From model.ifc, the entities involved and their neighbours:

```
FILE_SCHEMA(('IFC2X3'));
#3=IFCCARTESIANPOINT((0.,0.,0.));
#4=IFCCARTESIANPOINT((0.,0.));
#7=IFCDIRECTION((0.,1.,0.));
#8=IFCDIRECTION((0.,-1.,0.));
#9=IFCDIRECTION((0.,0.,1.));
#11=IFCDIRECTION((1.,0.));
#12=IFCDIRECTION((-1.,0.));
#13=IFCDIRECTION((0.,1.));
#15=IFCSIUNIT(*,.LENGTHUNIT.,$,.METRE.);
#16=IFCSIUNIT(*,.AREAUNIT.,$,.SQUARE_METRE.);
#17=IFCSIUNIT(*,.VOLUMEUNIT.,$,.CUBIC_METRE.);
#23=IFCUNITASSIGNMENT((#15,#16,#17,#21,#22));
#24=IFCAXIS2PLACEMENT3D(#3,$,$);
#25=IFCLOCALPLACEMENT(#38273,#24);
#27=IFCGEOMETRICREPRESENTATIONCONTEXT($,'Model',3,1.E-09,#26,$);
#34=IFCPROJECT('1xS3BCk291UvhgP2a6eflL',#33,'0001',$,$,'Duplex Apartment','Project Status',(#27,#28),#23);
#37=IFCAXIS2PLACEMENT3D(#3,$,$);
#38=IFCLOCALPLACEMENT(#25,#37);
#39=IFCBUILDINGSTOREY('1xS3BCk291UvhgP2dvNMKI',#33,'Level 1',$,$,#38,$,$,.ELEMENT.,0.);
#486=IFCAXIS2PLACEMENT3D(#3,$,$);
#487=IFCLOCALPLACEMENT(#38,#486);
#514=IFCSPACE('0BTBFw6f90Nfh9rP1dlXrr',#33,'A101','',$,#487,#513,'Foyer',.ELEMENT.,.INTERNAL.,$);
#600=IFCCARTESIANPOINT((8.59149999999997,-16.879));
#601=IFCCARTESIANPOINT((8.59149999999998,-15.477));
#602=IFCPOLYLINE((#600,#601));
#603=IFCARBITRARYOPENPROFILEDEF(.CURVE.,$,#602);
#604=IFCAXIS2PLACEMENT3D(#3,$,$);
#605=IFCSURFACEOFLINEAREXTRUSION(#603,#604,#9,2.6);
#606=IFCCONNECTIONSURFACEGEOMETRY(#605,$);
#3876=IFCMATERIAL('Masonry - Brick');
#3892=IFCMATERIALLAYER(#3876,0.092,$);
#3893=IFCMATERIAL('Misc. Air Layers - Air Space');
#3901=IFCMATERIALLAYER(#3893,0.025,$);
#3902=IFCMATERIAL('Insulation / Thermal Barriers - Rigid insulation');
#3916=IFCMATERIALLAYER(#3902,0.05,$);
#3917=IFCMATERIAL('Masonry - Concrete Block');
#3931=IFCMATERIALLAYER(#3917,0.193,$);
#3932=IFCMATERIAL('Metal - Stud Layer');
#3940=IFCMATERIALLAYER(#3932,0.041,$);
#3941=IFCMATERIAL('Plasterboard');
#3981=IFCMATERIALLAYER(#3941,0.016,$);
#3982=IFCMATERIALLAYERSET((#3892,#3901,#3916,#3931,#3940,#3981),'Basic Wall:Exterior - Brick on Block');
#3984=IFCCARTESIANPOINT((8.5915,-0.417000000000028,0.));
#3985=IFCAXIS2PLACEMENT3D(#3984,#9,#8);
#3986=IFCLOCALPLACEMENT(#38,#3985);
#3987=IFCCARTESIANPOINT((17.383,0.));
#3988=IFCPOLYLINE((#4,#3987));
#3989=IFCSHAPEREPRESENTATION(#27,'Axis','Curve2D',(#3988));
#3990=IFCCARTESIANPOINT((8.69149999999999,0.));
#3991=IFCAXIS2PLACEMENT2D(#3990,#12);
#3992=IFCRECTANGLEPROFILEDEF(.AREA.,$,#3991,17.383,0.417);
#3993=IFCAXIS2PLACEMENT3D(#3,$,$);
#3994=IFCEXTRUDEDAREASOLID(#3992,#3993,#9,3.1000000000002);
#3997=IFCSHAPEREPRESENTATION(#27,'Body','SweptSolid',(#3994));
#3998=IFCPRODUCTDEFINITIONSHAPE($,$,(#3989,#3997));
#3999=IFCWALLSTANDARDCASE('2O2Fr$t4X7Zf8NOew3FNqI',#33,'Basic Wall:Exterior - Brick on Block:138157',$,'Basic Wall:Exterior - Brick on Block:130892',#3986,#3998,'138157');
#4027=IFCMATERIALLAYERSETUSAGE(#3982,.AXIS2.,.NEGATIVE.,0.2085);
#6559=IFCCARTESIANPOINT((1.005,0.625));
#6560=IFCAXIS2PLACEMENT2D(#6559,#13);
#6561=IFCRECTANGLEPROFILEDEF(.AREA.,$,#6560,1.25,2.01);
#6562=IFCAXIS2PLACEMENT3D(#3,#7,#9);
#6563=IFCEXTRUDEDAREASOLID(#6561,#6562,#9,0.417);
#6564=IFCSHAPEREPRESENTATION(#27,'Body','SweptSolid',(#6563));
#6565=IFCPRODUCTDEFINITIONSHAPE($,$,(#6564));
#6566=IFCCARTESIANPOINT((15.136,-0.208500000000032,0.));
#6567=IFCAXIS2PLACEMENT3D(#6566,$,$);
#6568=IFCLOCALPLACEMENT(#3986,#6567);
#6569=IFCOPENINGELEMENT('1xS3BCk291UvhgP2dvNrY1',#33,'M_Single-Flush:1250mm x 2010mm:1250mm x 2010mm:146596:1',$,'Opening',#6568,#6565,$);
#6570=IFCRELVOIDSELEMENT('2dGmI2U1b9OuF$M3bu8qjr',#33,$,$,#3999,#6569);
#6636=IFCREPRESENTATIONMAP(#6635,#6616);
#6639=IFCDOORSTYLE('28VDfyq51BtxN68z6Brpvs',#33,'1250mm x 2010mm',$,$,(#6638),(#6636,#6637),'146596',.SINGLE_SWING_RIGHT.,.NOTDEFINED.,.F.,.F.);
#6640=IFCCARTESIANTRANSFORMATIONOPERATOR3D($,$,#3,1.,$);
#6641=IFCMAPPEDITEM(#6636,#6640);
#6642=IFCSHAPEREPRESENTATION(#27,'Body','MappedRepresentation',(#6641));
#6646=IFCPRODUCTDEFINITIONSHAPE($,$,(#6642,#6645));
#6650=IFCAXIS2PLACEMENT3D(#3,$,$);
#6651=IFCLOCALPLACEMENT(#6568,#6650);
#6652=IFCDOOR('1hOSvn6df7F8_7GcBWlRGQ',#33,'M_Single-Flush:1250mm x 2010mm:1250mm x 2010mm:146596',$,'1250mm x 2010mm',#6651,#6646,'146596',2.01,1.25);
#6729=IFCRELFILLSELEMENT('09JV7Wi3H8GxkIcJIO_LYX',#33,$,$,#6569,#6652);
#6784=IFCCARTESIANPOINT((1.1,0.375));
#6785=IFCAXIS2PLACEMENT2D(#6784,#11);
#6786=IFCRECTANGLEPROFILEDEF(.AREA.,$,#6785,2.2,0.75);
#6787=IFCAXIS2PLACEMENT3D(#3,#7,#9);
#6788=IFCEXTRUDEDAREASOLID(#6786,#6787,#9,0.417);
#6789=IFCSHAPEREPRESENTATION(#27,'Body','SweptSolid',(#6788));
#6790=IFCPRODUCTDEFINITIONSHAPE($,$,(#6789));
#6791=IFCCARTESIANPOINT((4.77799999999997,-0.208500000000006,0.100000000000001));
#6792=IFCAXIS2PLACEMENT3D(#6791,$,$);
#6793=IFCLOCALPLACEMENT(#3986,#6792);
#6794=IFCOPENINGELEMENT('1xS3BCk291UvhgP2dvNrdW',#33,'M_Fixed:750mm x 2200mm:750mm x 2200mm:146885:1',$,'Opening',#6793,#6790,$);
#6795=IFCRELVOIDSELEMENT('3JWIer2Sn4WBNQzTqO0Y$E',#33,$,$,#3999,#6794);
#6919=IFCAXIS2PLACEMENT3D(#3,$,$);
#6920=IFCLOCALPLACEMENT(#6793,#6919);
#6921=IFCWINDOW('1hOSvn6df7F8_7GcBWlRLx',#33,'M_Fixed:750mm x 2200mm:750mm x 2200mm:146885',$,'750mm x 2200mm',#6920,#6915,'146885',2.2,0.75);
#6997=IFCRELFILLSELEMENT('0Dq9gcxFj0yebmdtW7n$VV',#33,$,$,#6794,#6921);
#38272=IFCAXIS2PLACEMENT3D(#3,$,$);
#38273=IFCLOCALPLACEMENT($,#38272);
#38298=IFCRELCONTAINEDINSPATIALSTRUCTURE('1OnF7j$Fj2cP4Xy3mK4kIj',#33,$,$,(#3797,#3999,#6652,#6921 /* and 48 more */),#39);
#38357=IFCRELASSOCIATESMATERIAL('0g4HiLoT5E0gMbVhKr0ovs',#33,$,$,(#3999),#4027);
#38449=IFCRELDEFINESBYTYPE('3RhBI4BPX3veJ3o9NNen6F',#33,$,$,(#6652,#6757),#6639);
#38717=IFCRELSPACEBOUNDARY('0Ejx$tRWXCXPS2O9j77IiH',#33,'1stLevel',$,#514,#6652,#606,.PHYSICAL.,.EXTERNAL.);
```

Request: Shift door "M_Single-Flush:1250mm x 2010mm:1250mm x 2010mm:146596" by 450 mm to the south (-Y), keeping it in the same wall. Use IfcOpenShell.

```python
import numpy as np
import ifcopenshell
import ifcopenshell.api.geometry
import ifcopenshell.util.placement

model = ifcopenshell.open("model.ifc")

door = model.by_guid("1hOSvn6df7F8_7GcBWlRGQ")
opening = door.FillsVoids[0].RelatingOpeningElement
wall = opening.VoidsElements[0].RelatingBuildingElement

wall_matrix = ifcopenshell.util.placement.get_local_placement(wall.ObjectPlacement)
shift = wall_matrix[:3, 0] * 0.45
before = ifcopenshell.util.placement.get_local_placement(door.ObjectPlacement)[:3, 3].copy()

# The door is placed relative to its opening, so it follows when the opening moves.
matrix = ifcopenshell.util.placement.get_local_placement(opening.ObjectPlacement)
matrix[:3, 3] += shift
ifcopenshell.api.geometry.edit_object_placement(
    model, product=opening, matrix=matrix, is_si=False, should_transform_children=True
)

# Space boundary surfaces are stored in each space's coordinates; move them too.
for rel in door.ProvidesBoundaries:
    if not rel.ConnectionGeometry:
        continue
    surface = rel.ConnectionGeometry.SurfaceOnRelatingElement
    space_matrix = ifcopenshell.util.placement.get_local_placement(rel.RelatingSpace.ObjectPlacement)
    point = np.array(surface.Position.Location.Coordinates) + space_matrix[:3, :3].T @ shift
    surface.Position = model.createIfcAxis2Placement3D(
        model.createIfcCartesianPoint(point.tolist()), surface.Position.Axis, surface.Position.RefDirection
    )

after = ifcopenshell.util.placement.get_local_placement(door.ObjectPlacement)[:3, 3]
print("door moved by", (after - before).round(3) + 0.0)

model.write("model_v2.ifc")
```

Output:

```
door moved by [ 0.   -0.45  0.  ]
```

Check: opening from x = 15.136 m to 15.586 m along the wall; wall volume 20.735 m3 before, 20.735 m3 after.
